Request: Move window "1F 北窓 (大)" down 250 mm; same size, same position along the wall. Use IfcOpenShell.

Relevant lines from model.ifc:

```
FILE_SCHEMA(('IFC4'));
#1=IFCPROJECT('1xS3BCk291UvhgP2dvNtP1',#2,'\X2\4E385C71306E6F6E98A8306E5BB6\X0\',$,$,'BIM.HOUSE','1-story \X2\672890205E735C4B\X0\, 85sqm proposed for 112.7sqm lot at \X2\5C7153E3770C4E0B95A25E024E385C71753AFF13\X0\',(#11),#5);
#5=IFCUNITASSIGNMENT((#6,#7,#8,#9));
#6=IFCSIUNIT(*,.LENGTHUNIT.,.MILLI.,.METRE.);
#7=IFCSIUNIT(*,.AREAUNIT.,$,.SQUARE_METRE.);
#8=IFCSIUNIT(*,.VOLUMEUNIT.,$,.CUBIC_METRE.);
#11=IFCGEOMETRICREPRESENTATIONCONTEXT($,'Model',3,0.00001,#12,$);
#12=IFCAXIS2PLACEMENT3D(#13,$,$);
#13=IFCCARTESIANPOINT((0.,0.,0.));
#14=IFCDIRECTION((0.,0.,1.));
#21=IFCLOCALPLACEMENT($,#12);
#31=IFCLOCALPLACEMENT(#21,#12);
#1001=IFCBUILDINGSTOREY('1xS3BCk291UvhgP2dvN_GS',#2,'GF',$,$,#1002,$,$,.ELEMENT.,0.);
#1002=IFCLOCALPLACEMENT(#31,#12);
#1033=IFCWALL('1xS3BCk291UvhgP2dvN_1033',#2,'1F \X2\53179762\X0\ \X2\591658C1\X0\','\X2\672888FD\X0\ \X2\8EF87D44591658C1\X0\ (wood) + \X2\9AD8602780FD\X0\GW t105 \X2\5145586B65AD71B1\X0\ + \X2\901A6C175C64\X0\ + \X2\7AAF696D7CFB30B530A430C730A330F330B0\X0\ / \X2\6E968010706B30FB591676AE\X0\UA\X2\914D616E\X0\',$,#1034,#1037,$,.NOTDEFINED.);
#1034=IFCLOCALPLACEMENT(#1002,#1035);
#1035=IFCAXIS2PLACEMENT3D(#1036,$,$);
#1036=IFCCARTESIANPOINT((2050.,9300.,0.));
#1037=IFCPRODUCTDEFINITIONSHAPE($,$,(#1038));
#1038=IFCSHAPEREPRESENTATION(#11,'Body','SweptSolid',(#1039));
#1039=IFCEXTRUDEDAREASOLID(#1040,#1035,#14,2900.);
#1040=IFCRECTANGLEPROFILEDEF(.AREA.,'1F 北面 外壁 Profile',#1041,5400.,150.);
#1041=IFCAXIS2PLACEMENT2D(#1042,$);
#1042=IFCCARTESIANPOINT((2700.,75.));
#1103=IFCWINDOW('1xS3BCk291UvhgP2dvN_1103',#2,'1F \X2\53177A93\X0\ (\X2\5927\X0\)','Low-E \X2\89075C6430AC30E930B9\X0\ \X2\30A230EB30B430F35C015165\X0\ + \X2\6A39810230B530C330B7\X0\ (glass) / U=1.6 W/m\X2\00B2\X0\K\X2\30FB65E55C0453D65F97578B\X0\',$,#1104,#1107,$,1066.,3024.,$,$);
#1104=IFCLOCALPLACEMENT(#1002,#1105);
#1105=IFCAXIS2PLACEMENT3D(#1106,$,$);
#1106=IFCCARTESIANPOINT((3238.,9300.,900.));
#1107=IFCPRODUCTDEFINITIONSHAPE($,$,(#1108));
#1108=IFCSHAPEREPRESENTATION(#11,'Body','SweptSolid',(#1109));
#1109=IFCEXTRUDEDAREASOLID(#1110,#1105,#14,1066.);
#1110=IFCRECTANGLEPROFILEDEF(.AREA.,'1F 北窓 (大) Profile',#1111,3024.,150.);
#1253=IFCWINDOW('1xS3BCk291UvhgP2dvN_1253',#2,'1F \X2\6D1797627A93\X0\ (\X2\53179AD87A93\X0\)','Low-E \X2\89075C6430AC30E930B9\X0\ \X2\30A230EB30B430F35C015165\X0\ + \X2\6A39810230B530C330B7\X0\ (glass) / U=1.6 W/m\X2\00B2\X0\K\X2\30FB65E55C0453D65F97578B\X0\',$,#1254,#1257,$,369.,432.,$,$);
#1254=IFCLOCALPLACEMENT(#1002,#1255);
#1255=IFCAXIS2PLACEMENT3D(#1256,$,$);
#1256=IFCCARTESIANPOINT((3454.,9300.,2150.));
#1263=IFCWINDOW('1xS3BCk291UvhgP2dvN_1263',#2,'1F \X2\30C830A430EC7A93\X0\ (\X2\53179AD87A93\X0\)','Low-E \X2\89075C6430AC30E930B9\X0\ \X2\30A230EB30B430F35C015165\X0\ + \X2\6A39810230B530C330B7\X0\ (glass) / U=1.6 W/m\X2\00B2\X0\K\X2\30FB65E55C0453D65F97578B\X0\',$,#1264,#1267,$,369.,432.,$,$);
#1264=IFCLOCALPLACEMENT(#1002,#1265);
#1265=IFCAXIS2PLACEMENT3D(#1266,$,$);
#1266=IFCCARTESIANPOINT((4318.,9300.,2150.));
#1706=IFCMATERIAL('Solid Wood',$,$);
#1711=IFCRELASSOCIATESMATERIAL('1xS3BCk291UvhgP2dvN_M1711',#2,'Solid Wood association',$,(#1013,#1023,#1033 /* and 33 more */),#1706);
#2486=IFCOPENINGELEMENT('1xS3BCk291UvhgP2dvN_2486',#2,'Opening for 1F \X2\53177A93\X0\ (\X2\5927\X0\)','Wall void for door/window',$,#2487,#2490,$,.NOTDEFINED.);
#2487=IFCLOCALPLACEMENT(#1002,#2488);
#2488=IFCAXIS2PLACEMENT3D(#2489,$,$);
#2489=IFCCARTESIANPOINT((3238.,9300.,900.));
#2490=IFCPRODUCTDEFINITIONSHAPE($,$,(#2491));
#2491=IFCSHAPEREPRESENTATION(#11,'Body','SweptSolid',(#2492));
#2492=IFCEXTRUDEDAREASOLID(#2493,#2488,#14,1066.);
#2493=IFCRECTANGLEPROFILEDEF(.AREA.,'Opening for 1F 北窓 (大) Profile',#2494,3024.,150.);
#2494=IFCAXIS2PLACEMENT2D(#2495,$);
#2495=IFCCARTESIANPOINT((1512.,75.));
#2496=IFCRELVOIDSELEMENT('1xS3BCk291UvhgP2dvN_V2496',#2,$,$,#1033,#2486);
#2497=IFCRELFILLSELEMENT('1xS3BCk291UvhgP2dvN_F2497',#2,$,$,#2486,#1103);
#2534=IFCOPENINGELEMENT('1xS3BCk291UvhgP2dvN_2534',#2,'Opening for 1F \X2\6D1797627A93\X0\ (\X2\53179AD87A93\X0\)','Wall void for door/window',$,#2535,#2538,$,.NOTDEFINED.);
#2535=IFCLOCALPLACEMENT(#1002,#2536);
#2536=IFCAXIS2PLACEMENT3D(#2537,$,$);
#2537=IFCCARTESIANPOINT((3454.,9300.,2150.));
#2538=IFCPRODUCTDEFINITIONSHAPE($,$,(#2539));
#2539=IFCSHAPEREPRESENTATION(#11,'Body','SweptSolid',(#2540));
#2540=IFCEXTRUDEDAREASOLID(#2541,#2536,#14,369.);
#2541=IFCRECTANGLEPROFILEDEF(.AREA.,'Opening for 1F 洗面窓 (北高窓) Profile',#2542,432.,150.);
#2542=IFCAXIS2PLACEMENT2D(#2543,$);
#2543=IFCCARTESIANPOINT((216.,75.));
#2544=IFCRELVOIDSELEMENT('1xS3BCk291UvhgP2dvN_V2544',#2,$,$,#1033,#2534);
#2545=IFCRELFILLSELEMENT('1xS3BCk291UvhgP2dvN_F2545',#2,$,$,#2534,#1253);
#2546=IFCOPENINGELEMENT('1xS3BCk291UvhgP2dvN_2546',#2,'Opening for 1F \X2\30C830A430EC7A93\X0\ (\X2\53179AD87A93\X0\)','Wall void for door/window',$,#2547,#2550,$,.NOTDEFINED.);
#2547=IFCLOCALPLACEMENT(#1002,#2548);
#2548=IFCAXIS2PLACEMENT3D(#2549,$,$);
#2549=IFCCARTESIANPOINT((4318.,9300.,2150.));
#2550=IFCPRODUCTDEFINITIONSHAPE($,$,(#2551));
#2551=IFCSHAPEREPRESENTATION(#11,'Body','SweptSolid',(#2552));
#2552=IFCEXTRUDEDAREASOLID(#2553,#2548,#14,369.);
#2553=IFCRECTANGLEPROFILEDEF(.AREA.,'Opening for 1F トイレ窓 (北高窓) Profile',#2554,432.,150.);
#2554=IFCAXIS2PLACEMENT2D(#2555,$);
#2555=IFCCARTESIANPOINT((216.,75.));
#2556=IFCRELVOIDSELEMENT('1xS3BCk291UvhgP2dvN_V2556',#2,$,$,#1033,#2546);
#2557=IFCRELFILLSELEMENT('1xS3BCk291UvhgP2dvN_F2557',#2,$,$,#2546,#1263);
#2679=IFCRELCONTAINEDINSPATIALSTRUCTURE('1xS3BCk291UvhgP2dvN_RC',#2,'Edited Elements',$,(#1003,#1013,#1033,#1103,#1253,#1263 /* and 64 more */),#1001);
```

```python
import numpy as np
import ifcopenshell
import ifcopenshell.api.geometry
import ifcopenshell.util.placement
import ifcopenshell.util.unit

model = ifcopenshell.open("model.ifc")
unit_scale = ifcopenshell.util.unit.calculate_unit_scale(model)

window = model.by_id(1103)
opening = window.FillsVoids[0].RelatingOpeningElement
dz = -0.25 / unit_scale

shift = np.array([0.0, 0.0, dz])
# The window is not placed relative to its opening, so move both.
for product in (opening, window):
    matrix = ifcopenshell.util.placement.get_local_placement(product.ObjectPlacement)
    matrix[:3, 3] += shift
    ifcopenshell.api.geometry.edit_object_placement(model, product=product, matrix=matrix, is_si=False)

print(f"moved by {dz * unit_scale:+.3f} m")

model.write("model_edited.ifc")
```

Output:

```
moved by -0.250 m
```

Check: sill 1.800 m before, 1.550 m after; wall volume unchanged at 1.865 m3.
